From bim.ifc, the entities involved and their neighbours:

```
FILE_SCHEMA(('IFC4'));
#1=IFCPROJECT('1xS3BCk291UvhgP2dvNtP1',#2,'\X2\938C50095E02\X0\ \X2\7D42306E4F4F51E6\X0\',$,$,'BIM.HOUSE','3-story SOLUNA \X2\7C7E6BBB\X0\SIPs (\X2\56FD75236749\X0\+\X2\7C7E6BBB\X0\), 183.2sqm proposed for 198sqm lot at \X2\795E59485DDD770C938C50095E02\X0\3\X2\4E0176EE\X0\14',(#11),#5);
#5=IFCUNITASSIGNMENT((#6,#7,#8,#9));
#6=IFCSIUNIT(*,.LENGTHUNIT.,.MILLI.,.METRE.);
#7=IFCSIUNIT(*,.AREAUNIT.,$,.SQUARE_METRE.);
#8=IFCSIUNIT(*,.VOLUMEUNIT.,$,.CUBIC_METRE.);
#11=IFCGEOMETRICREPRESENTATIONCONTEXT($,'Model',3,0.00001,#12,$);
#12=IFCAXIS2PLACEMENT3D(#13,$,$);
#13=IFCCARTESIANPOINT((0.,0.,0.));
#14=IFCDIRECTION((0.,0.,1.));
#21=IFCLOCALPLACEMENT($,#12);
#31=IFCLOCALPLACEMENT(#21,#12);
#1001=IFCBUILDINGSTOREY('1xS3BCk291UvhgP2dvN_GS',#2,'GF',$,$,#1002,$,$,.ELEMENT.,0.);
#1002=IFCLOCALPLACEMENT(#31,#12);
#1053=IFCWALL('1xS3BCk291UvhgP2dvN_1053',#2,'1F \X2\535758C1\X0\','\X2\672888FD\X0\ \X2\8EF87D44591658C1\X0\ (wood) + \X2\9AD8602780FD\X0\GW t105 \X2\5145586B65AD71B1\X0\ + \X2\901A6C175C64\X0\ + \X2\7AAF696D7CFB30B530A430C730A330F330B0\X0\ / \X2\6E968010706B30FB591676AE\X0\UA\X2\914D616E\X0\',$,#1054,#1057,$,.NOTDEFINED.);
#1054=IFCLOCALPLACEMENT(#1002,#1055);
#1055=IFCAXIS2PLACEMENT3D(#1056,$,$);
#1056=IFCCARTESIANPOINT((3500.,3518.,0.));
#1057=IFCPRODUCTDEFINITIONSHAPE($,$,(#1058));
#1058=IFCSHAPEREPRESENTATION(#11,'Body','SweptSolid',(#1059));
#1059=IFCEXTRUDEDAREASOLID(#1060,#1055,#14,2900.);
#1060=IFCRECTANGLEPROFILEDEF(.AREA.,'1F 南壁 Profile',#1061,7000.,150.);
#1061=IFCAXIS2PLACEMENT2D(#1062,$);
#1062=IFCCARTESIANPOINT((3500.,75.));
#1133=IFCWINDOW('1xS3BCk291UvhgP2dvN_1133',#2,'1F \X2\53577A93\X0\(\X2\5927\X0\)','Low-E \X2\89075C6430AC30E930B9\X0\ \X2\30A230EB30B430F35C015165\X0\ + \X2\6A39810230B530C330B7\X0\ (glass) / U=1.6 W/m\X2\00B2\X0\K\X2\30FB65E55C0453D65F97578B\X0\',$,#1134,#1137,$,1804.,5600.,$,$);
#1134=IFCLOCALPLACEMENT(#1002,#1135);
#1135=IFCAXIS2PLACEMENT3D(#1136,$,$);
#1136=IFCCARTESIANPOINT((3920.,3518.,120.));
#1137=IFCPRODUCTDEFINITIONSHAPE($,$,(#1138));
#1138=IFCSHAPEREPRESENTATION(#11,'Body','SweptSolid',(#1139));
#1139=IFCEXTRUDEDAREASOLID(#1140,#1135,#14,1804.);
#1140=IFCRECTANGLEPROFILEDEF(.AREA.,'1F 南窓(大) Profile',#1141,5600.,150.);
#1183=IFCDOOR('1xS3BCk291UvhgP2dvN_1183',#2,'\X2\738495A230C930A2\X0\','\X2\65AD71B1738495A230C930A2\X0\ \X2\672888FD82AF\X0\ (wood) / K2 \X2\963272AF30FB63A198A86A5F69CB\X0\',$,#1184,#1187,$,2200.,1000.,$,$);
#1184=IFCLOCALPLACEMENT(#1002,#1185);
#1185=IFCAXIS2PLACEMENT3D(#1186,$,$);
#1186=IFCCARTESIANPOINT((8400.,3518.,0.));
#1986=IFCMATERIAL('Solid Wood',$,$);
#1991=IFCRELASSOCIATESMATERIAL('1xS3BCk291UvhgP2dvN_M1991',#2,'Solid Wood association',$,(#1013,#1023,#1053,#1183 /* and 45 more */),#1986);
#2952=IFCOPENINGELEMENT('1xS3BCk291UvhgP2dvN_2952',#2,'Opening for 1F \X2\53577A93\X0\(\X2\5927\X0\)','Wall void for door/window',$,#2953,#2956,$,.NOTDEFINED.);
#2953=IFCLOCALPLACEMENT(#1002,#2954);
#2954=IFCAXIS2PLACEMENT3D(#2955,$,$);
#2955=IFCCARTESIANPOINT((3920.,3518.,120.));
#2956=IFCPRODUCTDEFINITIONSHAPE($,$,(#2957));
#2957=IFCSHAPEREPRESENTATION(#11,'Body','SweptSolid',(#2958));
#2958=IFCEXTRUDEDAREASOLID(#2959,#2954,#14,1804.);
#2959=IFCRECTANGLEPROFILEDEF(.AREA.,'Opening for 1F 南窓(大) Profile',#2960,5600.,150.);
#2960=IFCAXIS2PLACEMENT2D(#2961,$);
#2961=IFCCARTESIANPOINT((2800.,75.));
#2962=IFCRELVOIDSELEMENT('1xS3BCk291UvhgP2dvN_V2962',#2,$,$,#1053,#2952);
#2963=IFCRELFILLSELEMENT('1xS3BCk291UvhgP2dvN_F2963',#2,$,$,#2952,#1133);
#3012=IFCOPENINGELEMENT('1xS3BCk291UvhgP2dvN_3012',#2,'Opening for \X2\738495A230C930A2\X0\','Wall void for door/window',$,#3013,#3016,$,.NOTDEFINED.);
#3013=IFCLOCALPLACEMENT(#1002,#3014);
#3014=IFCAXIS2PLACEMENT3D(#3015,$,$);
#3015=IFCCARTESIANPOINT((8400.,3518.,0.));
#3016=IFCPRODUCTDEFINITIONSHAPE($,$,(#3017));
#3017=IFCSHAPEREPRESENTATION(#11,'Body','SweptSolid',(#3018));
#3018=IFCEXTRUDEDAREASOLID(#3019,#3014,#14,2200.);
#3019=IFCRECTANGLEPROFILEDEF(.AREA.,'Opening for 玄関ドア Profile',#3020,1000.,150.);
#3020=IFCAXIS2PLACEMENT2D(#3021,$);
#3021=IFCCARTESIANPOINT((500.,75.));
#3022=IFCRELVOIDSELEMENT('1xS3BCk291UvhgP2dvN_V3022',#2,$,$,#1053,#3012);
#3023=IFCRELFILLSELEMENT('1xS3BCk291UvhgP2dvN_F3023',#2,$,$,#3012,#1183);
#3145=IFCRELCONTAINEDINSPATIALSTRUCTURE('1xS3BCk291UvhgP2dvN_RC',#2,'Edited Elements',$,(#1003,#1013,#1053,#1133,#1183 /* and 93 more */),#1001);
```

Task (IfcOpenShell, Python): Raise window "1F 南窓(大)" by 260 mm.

```python
import numpy as np
import ifcopenshell
import ifcopenshell.api.geometry
import ifcopenshell.util.placement
import ifcopenshell.util.unit

model = ifcopenshell.open("bim.ifc")
unit_scale = ifcopenshell.util.unit.calculate_unit_scale(model)

window = model.by_guid("1xS3BCk291UvhgP2dvN_1133")
opening = window.FillsVoids[0].RelatingOpeningElement
dz = 0.26 / unit_scale

shift = np.array([0.0, 0.0, dz])
# The window is not placed relative to its opening, so move both.
for product in (opening, window):
    matrix = ifcopenshell.util.placement.get_local_placement(product.ObjectPlacement)
    matrix[:3, 3] += shift
    ifcopenshell.api.geometry.edit_object_placement(model, product=product, matrix=matrix, is_si=False)

print(f"moved by {dz * unit_scale:+.3f} m")

model.write("bim_v2.ifc")
```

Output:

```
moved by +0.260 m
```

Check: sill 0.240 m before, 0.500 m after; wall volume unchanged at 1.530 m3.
